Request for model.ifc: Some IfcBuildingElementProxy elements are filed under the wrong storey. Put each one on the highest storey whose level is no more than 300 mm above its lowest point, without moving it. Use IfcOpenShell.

First a look at what the model holds.

```python
import ifcopenshell
import ifcopenshell.util.element
import ifcopenshell.util.placement

model = ifcopenshell.open("model.ifc")
print(model.schema)
for storey in model.by_type("IfcBuildingStorey"):
    level = ifcopenshell.util.placement.get_storey_elevation(storey)
    count = sum(e.is_a("IfcBuildingElementProxy") for e in ifcopenshell.util.element.get_contained(storey))
    print(storey.id(), storey.Name, round(level, 3), count, sep=" | ")
```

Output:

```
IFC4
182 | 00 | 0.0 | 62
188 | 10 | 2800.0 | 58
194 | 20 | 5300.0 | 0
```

```python
import ifcopenshell
import ifcopenshell.api.spatial
import ifcopenshell.geom
import ifcopenshell.util.element
import ifcopenshell.util.placement
import ifcopenshell.util.shape
import ifcopenshell.util.unit

model = ifcopenshell.open("model.ifc")
unit_scale = ifcopenshell.util.unit.calculate_unit_scale(model)
settings = ifcopenshell.geom.settings()

levels = sorted(
    ((ifcopenshell.util.placement.get_storey_elevation(s) * unit_scale, s) for s in model.by_type("IfcBuildingStorey")),
    key=lambda pair: pair[0],
)

for e in model.by_type("IfcBuildingElementProxy"):
    current = e.ContainedInStructure[0].RelatingStructure if e.ContainedInStructure else None
    if current is None or not current.is_a("IfcBuildingStorey"):
        continue
    shape = ifcopenshell.geom.create_shape(settings, e)
    bottom = ifcopenshell.util.shape.get_shape_bottom_elevation(shape, shape.geometry)
    below = [s for level, s in levels if level <= bottom + 0.3]
    storey = below[-1] if below else levels[0][1]
    if storey != current:
        # assign_container keeps the world position.
        ifcopenshell.api.spatial.assign_container(model, products=[e], relating_structure=storey)
        print(e.id(), current.Name, "->", storey.Name)

model.write("model-out.ifc")
```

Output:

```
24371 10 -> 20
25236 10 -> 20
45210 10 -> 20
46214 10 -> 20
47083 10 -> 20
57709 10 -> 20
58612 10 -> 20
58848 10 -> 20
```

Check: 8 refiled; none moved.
